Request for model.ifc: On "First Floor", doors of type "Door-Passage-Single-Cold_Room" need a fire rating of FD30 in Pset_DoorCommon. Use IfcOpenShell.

First a look at what the model holds.

```python
import ifcopenshell
import ifcopenshell.util.element

model = ifcopenshell.open("model.ifc")
print(model.schema)
storey = next(s for s in model.by_type("IfcBuildingStorey") if s.Name == "First Floor")
doors = [e for e in ifcopenshell.util.element.get_decomposition(storey) if e.is_a("IfcDoor")]
seen = {}
for e in doors:
    element_type = ifcopenshell.util.element.get_type(e)
    key = (element_type.Name if element_type != e and element_type else None, ifcopenshell.util.element.get_pset(e, "Pset_DoorCommon", "FireRating"))
    seen[key] = seen.get(key, 0) + 1
for (name, value), count in sorted(seen.items(), key=str):
    print(count, "x", name, "|", value)
```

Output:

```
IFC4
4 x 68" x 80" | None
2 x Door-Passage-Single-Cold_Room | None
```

```python
import ifcopenshell
import ifcopenshell.api.pset
import ifcopenshell.util.element

model = ifcopenshell.open("model.ifc")

storey = next(s for s in model.by_type("IfcBuildingStorey") if s.Name == "First Floor")
doors = [e for e in ifcopenshell.util.element.get_decomposition(storey) if e.is_a("IfcDoor")]

count = 0
for e in doors:
    element_type = ifcopenshell.util.element.get_type(e)
    if element_type in (None, e) or element_type.Name != "Door-Passage-Single-Cold_Room":
        continue
    # add_pset returns the element's existing set when there is one.
    pset = ifcopenshell.api.pset.add_pset(model, product=e, name="Pset_DoorCommon")
    ifcopenshell.api.pset.edit_pset(model, pset=pset, properties={"FireRating": "FD30"})
    count += 1

print(count, "doors updated")

model.write("model_rev.ifc")
```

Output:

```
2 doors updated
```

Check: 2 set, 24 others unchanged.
